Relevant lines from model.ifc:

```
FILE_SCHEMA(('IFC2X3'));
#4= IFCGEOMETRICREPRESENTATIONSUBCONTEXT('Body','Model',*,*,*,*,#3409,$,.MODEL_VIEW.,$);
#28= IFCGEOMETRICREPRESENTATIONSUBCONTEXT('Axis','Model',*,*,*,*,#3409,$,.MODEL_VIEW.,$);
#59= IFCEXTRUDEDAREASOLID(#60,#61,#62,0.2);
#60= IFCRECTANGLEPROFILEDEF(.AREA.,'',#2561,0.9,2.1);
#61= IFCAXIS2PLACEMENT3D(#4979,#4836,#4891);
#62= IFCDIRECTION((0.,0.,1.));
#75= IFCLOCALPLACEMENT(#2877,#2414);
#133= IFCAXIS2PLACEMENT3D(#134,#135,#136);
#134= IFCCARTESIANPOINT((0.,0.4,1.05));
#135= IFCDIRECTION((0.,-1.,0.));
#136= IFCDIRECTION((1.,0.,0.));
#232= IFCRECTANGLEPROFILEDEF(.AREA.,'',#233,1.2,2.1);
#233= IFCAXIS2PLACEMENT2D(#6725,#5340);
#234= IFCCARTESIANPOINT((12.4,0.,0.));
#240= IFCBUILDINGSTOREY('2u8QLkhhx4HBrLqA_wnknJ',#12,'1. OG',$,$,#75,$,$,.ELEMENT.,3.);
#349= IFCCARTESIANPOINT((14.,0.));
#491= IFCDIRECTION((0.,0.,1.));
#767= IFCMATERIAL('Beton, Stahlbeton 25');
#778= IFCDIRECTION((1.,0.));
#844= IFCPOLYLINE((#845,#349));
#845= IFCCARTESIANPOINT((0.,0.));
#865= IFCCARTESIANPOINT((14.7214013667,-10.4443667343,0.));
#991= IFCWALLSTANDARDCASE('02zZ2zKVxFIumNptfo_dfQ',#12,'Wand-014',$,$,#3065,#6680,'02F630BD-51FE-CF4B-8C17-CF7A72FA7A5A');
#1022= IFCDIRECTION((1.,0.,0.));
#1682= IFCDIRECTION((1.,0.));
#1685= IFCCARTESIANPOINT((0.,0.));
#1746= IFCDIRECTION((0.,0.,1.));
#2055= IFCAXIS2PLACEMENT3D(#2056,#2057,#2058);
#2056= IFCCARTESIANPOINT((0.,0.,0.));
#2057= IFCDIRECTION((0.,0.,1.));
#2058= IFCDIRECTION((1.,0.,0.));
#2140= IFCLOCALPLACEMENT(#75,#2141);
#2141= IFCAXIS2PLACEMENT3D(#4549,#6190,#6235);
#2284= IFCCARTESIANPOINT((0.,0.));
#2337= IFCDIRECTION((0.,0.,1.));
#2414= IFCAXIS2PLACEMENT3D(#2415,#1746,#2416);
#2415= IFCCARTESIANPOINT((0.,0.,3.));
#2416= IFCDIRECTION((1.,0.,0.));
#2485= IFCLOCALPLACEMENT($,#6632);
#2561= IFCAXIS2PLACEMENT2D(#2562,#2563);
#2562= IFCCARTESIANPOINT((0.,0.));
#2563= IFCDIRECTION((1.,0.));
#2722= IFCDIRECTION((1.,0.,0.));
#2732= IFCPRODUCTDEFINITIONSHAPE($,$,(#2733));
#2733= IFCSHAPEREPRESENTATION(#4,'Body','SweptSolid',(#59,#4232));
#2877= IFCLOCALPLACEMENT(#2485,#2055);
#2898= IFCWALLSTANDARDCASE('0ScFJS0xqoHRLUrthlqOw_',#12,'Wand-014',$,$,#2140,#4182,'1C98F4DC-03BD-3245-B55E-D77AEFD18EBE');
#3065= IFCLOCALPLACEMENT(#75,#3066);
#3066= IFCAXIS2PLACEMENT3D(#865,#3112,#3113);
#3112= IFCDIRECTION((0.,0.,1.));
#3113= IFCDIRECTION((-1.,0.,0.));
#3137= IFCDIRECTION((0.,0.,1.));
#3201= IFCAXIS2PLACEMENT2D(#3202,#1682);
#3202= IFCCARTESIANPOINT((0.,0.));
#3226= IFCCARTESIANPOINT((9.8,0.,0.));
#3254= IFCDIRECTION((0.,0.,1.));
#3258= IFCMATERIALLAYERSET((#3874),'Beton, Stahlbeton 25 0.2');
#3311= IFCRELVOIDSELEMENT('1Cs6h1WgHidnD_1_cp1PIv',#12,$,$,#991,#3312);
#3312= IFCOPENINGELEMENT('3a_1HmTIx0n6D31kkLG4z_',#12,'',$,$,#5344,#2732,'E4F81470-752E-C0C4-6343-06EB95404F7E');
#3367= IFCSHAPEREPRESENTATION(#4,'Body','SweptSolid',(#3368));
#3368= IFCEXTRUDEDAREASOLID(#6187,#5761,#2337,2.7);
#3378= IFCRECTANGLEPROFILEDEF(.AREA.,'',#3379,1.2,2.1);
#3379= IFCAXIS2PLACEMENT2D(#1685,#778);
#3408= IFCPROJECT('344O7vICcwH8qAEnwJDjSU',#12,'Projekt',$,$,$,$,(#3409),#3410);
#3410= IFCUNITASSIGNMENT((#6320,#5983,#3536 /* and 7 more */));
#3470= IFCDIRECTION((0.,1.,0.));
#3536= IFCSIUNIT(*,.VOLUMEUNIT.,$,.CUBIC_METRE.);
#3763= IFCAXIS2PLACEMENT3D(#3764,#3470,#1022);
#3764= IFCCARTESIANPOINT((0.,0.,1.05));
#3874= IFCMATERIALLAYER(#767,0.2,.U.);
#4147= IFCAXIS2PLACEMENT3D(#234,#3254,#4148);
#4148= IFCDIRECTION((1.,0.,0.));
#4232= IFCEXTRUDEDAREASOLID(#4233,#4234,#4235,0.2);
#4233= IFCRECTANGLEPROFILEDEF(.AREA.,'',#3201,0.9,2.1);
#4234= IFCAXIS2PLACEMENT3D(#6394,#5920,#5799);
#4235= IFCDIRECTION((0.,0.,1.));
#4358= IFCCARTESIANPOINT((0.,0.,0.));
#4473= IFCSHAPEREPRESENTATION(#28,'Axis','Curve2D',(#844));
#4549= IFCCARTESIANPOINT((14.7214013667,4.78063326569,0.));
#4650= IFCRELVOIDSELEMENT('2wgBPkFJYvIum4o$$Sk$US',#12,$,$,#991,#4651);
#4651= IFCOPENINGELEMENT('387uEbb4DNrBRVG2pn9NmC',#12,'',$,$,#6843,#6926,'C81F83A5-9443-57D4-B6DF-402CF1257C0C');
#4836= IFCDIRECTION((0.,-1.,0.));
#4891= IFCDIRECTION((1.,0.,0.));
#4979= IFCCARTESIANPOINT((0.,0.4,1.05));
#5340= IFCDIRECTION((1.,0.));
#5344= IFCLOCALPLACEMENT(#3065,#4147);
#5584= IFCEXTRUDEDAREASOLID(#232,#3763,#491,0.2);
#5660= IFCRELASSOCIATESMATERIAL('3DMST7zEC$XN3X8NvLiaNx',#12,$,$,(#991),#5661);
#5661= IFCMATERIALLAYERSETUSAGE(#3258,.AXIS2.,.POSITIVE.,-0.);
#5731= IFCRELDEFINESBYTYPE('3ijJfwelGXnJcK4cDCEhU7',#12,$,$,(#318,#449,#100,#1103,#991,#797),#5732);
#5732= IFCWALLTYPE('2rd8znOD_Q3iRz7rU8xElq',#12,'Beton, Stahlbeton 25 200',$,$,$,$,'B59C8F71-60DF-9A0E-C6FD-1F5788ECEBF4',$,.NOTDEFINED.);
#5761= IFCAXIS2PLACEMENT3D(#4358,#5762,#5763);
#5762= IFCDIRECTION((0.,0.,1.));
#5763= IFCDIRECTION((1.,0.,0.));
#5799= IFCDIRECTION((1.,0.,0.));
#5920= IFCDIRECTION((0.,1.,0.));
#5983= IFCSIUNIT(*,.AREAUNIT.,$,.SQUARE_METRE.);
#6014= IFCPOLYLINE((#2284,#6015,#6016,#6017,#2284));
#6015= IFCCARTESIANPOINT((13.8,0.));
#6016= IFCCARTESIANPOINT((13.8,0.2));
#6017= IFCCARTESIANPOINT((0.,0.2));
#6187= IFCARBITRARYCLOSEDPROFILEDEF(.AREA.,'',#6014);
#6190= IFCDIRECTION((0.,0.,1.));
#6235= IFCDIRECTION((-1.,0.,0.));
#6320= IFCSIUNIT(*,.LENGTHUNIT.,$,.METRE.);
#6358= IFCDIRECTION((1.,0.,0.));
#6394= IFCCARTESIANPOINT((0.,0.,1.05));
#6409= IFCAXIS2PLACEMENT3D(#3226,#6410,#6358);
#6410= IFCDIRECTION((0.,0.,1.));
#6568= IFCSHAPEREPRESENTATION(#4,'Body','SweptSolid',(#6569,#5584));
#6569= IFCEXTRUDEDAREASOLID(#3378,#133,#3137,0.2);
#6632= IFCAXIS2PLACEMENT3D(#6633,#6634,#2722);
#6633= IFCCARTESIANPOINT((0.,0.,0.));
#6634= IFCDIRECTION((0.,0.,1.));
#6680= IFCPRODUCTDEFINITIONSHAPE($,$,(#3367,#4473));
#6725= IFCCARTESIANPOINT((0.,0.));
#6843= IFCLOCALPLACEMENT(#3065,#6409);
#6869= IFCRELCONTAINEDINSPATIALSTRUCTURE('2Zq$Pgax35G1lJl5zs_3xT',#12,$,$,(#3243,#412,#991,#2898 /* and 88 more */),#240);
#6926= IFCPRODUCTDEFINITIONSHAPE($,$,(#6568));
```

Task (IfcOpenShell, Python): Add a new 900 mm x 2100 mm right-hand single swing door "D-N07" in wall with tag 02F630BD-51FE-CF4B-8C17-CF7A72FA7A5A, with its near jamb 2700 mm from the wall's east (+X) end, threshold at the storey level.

```python
import numpy as np
import ifcopenshell
import ifcopenshell.api.feature
import ifcopenshell.api.geometry
import ifcopenshell.api.root
import ifcopenshell.api.spatial
import ifcopenshell.api.type
import ifcopenshell.geom
import ifcopenshell.util.element
import ifcopenshell.util.placement
import ifcopenshell.util.representation
import ifcopenshell.util.shape
import ifcopenshell.util.unit

model = ifcopenshell.open("model.ifc")
unit_scale = ifcopenshell.util.unit.calculate_unit_scale(model)
settings = ifcopenshell.geom.settings()


def volume(element):
    """Net volume in cubic metres, openings subtracted."""
    shape = ifcopenshell.geom.create_shape(settings, element)
    return ifcopenshell.util.shape.get_volume(shape.geometry)


wall = model.by_guid("02zZ2zKVxFIumNptfo_dfQ")
storey = ifcopenshell.util.element.get_container(wall, ifc_class="IfcBuildingStorey")
context = ifcopenshell.util.representation.get_context(model, "Model", "Body", "MODEL_VIEW")
before = volume(wall)

width, height, from_end, sill = 0.9, 2.1, 2.7, 0.0  # metres

# The wall runs along its own X axis, and the end named is its -X end.
wall_shape = ifcopenshell.geom.create_shape(settings, wall)
x, y, z = ifcopenshell.util.shape.get_vertices(wall_shape.geometry).T
start = x.min() + from_end
face, thickness = float(y.min()), float(y.max() - y.min())
wall_matrix = ifcopenshell.util.placement.get_local_placement(wall.ObjectPlacement)
level = ifcopenshell.util.placement.get_local_placement(storey.ObjectPlacement)[2, 3]


def in_wall(x, y):
    """Placement at x, y metres in the wall's axes, at sill height."""
    matrix = wall_matrix.copy()
    matrix[:, 3] = wall_matrix @ np.array([x / unit_scale, y / unit_scale, 0.0, 1.0])
    matrix[2, 3] = level + sill / unit_scale
    return matrix


# Opening: a box that overshoots both wall faces by 50 mm.
opening = ifcopenshell.api.root.create_entity(model, ifc_class="IfcOpeningElement")
box = ifcopenshell.api.geometry.add_wall_representation(
    model, context=context, length=width, height=height, thickness=thickness + 0.1
)
ifcopenshell.api.geometry.assign_representation(model, product=opening, representation=box)
ifcopenshell.api.geometry.edit_object_placement(model, product=opening, matrix=in_wall(start, face - 0.05), is_si=False)
ifcopenshell.api.feature.add_feature(model, feature=opening, element=wall)

door = ifcopenshell.api.root.create_entity(model, ifc_class="IfcDoor", name="D-N07")
door.OverallWidth, door.OverallHeight = width / unit_scale, height / unit_scale
body = ifcopenshell.api.geometry.add_door_representation(
    model,
    context=context,
    overall_width=door.OverallWidth,
    overall_height=door.OverallHeight,
    operation_type="SINGLE_SWING_RIGHT",
    lining_properties={"LiningDepth": thickness / unit_scale, "ThresholdDepth": thickness / unit_scale},
)
ifcopenshell.api.geometry.assign_representation(model, product=door, representation=body)
ifcopenshell.api.spatial.assign_container(model, products=[door], relating_structure=storey)
fills = ifcopenshell.api.feature.add_filling(model, opening=opening, element=door)
fills.OwnerHistory = door.OwnerHistory  # required in IFC2X3

# IFC2X3 keeps the operation on the door style.
style = ifcopenshell.api.root.create_entity(model, ifc_class="IfcDoorStyle", name="D-N07")
style.OperationType, style.ConstructionType = "SINGLE_SWING_RIGHT", "NOTDEFINED"
style.ParameterTakesPrecedence = style.Sizeable = False
ifcopenshell.api.type.assign_type(model, related_objects=[door], relating_type=style)

# The lining spans the wall, so the door starts at the wall face.
ifcopenshell.api.geometry.edit_object_placement(model, product=door, matrix=in_wall(start, face), is_si=False)

after = volume(wall)

print(f"wall volume {before:.3f} -> {after:.3f} m3")

model.write("model_rev.ifc")
```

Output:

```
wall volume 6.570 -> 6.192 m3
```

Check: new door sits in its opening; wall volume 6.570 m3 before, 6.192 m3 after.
